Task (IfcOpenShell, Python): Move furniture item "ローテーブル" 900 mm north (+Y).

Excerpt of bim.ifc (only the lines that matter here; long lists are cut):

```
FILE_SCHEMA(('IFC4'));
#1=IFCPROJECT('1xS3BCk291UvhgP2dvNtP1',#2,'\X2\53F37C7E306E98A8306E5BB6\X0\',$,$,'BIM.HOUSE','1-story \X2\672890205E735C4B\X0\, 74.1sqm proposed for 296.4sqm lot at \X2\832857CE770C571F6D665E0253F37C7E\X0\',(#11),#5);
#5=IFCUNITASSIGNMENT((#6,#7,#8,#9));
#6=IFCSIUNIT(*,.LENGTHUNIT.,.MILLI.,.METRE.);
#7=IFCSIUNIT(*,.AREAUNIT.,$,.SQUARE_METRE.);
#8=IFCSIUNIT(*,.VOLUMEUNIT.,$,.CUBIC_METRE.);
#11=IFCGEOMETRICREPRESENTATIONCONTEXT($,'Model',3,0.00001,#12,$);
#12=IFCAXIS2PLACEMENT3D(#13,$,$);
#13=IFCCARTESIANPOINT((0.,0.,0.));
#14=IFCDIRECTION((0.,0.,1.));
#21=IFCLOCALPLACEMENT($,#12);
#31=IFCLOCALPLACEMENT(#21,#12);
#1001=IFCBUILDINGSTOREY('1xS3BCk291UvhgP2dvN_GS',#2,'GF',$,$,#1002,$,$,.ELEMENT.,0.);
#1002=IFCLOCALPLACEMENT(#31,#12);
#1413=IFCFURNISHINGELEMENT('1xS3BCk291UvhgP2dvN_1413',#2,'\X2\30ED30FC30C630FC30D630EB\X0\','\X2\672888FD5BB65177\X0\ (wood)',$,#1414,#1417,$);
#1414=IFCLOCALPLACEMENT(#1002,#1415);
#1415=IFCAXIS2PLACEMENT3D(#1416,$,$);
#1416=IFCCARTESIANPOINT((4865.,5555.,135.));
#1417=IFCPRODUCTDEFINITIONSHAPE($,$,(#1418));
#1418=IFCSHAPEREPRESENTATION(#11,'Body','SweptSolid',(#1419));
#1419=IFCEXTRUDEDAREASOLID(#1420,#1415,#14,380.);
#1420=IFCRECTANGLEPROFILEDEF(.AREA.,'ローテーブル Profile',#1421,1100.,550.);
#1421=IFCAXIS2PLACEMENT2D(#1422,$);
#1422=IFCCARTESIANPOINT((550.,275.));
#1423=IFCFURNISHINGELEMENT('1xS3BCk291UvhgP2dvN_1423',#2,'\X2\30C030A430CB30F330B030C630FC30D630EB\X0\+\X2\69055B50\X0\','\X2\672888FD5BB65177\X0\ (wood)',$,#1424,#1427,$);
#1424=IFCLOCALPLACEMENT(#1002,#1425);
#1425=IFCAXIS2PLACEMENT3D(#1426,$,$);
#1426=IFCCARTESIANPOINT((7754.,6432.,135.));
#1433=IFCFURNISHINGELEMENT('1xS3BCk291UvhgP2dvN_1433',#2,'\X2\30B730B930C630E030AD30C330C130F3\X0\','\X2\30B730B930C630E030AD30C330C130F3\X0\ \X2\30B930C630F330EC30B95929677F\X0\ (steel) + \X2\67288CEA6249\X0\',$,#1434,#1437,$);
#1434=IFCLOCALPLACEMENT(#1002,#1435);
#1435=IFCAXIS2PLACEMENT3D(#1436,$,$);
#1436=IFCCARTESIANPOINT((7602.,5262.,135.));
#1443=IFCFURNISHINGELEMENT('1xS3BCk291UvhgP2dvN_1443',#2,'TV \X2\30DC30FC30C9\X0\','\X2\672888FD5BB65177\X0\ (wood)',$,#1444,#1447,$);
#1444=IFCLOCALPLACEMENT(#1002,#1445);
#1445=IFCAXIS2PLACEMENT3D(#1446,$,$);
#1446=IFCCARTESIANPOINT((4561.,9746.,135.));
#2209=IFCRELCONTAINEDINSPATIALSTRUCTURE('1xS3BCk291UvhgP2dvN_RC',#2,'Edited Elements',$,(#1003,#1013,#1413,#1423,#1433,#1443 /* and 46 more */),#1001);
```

```python
import ifcopenshell
import ifcopenshell.api.geometry
import ifcopenshell.util.placement

model = ifcopenshell.open("bim.ifc")

item = model.by_guid("1xS3BCk291UvhgP2dvN_1413")
matrix = ifcopenshell.util.placement.get_local_placement(item.ObjectPlacement)
matrix[1, 3] += 900.0
ifcopenshell.api.geometry.edit_object_placement(model, product=item, matrix=matrix, is_si=False)

print(ifcopenshell.util.placement.get_local_placement(item.ObjectPlacement).round(3) + 0.0)

model.write("bim_rev.ifc")
```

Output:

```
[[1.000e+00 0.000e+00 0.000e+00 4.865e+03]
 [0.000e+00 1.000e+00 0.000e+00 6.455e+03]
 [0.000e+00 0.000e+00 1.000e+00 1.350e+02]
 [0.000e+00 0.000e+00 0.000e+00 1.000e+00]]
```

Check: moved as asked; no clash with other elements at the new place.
